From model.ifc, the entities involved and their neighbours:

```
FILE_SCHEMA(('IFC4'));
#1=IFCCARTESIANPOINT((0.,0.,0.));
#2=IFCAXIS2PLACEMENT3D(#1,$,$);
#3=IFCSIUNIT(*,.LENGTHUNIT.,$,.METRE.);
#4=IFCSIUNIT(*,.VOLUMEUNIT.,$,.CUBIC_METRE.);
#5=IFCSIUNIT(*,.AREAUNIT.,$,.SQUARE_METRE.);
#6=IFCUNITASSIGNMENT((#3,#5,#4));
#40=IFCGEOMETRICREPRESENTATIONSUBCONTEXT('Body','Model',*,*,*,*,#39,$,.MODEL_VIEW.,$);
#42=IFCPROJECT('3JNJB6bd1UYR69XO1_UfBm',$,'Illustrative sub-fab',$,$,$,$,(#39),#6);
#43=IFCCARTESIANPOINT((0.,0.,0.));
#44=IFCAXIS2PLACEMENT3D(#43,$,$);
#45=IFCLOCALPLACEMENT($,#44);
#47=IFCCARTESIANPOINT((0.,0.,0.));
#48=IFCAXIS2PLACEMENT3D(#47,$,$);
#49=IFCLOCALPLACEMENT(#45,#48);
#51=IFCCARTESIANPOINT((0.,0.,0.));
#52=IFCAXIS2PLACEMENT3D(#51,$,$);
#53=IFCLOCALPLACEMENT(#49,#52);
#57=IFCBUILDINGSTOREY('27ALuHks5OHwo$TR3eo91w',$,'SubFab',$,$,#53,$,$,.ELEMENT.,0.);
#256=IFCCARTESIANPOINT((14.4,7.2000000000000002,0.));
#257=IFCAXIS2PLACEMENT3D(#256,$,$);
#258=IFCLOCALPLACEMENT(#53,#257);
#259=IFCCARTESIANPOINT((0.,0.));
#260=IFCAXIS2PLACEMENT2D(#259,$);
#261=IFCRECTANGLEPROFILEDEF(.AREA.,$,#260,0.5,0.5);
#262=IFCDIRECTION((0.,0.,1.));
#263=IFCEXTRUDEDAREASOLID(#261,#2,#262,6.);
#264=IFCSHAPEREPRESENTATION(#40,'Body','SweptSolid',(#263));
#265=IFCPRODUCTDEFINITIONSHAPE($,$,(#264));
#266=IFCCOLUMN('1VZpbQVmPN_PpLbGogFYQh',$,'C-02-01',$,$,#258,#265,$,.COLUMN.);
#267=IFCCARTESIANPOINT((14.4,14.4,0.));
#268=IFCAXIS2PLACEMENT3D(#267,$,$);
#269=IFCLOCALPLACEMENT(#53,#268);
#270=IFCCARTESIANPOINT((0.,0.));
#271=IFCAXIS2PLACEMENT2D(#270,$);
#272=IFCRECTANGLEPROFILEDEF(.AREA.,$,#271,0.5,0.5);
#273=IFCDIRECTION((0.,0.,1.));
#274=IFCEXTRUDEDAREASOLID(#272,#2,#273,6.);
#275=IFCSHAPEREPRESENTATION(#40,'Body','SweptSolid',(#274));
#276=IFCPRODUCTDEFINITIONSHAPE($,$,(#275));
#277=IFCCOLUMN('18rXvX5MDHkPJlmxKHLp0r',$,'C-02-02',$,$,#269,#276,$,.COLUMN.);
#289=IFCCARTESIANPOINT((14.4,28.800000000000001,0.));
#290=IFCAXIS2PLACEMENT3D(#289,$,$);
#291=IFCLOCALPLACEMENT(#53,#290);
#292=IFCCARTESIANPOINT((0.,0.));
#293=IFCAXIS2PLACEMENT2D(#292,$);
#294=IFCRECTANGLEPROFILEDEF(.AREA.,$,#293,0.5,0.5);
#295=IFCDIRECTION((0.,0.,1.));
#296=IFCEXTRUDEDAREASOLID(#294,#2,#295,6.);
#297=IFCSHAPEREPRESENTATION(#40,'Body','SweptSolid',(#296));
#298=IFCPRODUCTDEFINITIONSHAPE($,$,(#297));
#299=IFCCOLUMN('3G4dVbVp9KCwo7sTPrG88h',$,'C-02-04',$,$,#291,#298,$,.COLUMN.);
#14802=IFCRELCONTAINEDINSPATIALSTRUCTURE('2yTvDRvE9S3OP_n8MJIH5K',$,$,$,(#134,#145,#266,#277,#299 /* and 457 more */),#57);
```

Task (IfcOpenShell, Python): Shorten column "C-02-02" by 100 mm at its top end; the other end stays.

```python
import ifcopenshell
import ifcopenshell.util.representation
import ifcopenshell.util.unit

model = ifcopenshell.open("model.ifc")
unit_scale = ifcopenshell.util.unit.calculate_unit_scale(model)

member = model.by_guid("18rXvX5MDHkPJlmxKHLp0r")
change = -0.1 / unit_scale

# The extrusion runs towards the end named, so only its depth changes.
body = ifcopenshell.util.representation.get_representation(member, "Model", "Body")
solid = body.Items[0]
old_length = solid.Depth
solid.Depth += change

print(f"length {old_length:g} -> {solid.Depth:g}")

model.write("model-out.ifc")
```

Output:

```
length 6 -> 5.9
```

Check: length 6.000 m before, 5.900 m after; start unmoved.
